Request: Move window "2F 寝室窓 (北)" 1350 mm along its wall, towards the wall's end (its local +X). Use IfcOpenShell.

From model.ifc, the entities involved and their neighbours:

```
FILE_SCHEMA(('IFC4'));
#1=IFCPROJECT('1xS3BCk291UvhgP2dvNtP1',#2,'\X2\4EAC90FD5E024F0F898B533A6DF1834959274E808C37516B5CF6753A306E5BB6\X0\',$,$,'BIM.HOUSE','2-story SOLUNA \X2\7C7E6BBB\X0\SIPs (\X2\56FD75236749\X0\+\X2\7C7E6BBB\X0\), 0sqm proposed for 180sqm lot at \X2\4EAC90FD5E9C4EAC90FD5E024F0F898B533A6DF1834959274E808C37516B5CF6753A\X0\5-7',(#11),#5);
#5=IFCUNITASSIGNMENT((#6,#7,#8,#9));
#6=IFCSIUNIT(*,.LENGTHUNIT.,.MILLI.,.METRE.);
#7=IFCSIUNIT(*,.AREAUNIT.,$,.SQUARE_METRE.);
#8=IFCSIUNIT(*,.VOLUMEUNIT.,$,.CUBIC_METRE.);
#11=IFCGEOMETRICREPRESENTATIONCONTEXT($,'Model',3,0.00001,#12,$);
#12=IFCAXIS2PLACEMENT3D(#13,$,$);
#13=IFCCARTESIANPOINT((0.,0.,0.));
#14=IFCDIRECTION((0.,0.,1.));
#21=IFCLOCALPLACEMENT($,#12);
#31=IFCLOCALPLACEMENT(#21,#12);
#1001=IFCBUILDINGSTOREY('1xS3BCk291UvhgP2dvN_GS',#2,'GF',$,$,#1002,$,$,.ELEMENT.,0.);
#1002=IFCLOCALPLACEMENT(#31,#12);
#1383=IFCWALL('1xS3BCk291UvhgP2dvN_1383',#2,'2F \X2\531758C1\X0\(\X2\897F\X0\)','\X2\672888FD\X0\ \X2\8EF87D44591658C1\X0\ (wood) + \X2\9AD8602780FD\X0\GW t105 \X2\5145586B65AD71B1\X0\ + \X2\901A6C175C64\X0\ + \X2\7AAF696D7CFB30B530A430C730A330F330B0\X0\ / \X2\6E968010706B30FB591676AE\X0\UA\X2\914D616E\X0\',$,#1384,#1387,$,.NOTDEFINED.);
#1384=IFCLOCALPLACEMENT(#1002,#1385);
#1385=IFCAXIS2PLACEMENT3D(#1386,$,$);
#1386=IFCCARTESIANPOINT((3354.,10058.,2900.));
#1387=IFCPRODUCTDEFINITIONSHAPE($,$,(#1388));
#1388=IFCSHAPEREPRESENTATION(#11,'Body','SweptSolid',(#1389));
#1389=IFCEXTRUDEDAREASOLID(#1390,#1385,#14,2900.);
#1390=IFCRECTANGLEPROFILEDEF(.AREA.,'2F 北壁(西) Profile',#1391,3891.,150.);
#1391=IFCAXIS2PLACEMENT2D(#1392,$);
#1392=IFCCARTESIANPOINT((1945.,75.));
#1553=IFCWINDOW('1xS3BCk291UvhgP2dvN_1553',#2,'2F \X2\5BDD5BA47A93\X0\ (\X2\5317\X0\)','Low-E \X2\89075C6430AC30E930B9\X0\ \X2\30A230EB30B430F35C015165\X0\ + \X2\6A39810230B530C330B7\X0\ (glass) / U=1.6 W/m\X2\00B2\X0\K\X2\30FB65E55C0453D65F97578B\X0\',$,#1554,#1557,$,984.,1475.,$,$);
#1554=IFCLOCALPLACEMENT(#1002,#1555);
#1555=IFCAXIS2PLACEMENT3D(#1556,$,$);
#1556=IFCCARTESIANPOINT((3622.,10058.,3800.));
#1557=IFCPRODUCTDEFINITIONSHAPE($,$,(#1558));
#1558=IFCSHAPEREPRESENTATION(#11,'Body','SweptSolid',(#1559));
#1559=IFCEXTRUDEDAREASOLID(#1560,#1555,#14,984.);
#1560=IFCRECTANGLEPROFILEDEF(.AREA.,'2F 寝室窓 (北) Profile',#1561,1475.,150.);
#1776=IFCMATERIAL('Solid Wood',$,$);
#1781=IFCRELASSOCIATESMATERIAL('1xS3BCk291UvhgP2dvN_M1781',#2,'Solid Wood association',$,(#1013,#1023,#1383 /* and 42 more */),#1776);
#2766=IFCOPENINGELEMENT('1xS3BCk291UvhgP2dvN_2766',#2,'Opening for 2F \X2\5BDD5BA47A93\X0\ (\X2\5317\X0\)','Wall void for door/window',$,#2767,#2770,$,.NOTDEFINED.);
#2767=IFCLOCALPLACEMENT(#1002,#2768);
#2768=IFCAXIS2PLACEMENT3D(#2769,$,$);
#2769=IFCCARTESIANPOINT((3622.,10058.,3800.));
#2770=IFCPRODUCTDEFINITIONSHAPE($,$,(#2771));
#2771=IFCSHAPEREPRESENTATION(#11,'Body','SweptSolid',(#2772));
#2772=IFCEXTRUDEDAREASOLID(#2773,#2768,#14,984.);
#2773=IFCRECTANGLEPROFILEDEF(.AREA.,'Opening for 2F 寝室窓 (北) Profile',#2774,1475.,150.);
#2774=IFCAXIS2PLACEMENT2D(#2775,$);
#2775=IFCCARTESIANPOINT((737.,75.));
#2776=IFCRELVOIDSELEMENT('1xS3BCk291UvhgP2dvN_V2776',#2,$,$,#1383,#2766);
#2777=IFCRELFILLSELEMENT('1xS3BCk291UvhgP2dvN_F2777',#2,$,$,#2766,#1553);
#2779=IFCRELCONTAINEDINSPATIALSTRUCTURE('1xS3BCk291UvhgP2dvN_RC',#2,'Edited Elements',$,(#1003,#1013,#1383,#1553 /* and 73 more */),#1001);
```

```python
import ifcopenshell
import ifcopenshell.api.geometry
import ifcopenshell.util.placement
import ifcopenshell.util.unit

model = ifcopenshell.open("model.ifc")
unit_scale = ifcopenshell.util.unit.calculate_unit_scale(model)

window = model.by_guid("1xS3BCk291UvhgP2dvN_1553")
opening = window.FillsVoids[0].RelatingOpeningElement
wall = opening.VoidsElements[0].RelatingBuildingElement

wall_matrix = ifcopenshell.util.placement.get_local_placement(wall.ObjectPlacement)
shift = wall_matrix[:3, 0] * 1.35 / unit_scale
before = ifcopenshell.util.placement.get_local_placement(window.ObjectPlacement)[:3, 3].copy()

# The window is not placed relative to its opening, so move both.
for product in (opening, window):
    matrix = ifcopenshell.util.placement.get_local_placement(product.ObjectPlacement)
    matrix[:3, 3] += shift
    ifcopenshell.api.geometry.edit_object_placement(model, product=product, matrix=matrix, is_si=False)

after = ifcopenshell.util.placement.get_local_placement(window.ObjectPlacement)[:3, 3]
print("window moved by", (after - before).round(3) + 0.0)

model.write("model_v2.ifc")
```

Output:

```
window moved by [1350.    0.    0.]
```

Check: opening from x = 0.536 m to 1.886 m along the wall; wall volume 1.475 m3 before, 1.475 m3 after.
